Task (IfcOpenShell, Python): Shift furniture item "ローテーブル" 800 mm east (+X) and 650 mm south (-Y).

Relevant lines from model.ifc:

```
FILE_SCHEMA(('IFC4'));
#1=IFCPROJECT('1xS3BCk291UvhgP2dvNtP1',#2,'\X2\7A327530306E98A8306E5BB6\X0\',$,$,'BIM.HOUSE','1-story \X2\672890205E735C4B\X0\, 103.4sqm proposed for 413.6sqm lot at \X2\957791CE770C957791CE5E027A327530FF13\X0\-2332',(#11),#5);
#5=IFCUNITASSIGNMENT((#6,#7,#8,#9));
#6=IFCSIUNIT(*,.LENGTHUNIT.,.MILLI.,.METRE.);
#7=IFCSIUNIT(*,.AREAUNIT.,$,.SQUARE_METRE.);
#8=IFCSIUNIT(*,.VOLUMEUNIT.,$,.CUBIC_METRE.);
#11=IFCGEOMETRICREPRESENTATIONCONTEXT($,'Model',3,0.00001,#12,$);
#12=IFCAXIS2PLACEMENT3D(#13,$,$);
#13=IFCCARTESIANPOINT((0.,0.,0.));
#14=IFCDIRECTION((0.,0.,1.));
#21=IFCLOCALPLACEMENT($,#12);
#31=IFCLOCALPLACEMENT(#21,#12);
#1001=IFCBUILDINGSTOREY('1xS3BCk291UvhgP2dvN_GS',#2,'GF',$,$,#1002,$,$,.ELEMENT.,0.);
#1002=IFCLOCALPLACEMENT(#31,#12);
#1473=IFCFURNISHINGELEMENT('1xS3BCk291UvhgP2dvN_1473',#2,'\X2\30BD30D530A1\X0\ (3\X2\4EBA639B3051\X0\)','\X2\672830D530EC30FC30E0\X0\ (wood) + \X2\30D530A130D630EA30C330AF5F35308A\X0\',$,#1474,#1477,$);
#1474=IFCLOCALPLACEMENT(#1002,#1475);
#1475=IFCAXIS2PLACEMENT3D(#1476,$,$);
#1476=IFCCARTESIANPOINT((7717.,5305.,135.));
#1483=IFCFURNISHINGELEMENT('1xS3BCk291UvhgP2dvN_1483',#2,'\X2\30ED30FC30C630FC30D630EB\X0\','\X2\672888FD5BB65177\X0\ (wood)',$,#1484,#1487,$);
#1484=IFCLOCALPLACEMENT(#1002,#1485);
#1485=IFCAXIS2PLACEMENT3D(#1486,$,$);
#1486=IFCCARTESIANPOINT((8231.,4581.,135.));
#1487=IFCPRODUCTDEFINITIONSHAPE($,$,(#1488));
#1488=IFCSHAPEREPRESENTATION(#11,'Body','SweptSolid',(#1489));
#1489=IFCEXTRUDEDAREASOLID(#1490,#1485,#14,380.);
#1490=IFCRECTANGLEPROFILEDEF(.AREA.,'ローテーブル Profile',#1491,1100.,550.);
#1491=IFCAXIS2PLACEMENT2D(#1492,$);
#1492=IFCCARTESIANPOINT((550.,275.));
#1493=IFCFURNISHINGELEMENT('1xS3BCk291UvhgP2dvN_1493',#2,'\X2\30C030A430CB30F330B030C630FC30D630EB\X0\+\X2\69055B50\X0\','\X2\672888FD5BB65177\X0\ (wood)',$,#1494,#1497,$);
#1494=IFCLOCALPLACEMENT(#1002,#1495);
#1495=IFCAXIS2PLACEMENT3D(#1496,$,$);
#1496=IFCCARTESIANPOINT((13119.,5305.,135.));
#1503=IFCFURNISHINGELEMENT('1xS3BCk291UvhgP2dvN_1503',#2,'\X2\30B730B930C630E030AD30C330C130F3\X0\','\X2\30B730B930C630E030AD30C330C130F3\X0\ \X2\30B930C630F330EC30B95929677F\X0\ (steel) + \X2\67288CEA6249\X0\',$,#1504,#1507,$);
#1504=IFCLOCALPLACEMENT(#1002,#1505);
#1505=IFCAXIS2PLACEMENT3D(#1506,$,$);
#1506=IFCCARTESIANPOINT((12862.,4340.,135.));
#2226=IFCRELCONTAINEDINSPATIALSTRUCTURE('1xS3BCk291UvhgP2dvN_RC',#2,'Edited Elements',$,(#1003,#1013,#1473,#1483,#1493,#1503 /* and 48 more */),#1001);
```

```python
import ifcopenshell
import ifcopenshell.api.geometry
import ifcopenshell.util.placement

model = ifcopenshell.open("model.ifc")

item = model.by_guid("1xS3BCk291UvhgP2dvN_1483")
matrix = ifcopenshell.util.placement.get_local_placement(item.ObjectPlacement)
matrix[0, 3] += 800.0
matrix[1, 3] -= 650.0
ifcopenshell.api.geometry.edit_object_placement(model, product=item, matrix=matrix, is_si=False)

print(ifcopenshell.util.placement.get_local_placement(item.ObjectPlacement).round(3) + 0.0)

model.write("model_v2.ifc")
```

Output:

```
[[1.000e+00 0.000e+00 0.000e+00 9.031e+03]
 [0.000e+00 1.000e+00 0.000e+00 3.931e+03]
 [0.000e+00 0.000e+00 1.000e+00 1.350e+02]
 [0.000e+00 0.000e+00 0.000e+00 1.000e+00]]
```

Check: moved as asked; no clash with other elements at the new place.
